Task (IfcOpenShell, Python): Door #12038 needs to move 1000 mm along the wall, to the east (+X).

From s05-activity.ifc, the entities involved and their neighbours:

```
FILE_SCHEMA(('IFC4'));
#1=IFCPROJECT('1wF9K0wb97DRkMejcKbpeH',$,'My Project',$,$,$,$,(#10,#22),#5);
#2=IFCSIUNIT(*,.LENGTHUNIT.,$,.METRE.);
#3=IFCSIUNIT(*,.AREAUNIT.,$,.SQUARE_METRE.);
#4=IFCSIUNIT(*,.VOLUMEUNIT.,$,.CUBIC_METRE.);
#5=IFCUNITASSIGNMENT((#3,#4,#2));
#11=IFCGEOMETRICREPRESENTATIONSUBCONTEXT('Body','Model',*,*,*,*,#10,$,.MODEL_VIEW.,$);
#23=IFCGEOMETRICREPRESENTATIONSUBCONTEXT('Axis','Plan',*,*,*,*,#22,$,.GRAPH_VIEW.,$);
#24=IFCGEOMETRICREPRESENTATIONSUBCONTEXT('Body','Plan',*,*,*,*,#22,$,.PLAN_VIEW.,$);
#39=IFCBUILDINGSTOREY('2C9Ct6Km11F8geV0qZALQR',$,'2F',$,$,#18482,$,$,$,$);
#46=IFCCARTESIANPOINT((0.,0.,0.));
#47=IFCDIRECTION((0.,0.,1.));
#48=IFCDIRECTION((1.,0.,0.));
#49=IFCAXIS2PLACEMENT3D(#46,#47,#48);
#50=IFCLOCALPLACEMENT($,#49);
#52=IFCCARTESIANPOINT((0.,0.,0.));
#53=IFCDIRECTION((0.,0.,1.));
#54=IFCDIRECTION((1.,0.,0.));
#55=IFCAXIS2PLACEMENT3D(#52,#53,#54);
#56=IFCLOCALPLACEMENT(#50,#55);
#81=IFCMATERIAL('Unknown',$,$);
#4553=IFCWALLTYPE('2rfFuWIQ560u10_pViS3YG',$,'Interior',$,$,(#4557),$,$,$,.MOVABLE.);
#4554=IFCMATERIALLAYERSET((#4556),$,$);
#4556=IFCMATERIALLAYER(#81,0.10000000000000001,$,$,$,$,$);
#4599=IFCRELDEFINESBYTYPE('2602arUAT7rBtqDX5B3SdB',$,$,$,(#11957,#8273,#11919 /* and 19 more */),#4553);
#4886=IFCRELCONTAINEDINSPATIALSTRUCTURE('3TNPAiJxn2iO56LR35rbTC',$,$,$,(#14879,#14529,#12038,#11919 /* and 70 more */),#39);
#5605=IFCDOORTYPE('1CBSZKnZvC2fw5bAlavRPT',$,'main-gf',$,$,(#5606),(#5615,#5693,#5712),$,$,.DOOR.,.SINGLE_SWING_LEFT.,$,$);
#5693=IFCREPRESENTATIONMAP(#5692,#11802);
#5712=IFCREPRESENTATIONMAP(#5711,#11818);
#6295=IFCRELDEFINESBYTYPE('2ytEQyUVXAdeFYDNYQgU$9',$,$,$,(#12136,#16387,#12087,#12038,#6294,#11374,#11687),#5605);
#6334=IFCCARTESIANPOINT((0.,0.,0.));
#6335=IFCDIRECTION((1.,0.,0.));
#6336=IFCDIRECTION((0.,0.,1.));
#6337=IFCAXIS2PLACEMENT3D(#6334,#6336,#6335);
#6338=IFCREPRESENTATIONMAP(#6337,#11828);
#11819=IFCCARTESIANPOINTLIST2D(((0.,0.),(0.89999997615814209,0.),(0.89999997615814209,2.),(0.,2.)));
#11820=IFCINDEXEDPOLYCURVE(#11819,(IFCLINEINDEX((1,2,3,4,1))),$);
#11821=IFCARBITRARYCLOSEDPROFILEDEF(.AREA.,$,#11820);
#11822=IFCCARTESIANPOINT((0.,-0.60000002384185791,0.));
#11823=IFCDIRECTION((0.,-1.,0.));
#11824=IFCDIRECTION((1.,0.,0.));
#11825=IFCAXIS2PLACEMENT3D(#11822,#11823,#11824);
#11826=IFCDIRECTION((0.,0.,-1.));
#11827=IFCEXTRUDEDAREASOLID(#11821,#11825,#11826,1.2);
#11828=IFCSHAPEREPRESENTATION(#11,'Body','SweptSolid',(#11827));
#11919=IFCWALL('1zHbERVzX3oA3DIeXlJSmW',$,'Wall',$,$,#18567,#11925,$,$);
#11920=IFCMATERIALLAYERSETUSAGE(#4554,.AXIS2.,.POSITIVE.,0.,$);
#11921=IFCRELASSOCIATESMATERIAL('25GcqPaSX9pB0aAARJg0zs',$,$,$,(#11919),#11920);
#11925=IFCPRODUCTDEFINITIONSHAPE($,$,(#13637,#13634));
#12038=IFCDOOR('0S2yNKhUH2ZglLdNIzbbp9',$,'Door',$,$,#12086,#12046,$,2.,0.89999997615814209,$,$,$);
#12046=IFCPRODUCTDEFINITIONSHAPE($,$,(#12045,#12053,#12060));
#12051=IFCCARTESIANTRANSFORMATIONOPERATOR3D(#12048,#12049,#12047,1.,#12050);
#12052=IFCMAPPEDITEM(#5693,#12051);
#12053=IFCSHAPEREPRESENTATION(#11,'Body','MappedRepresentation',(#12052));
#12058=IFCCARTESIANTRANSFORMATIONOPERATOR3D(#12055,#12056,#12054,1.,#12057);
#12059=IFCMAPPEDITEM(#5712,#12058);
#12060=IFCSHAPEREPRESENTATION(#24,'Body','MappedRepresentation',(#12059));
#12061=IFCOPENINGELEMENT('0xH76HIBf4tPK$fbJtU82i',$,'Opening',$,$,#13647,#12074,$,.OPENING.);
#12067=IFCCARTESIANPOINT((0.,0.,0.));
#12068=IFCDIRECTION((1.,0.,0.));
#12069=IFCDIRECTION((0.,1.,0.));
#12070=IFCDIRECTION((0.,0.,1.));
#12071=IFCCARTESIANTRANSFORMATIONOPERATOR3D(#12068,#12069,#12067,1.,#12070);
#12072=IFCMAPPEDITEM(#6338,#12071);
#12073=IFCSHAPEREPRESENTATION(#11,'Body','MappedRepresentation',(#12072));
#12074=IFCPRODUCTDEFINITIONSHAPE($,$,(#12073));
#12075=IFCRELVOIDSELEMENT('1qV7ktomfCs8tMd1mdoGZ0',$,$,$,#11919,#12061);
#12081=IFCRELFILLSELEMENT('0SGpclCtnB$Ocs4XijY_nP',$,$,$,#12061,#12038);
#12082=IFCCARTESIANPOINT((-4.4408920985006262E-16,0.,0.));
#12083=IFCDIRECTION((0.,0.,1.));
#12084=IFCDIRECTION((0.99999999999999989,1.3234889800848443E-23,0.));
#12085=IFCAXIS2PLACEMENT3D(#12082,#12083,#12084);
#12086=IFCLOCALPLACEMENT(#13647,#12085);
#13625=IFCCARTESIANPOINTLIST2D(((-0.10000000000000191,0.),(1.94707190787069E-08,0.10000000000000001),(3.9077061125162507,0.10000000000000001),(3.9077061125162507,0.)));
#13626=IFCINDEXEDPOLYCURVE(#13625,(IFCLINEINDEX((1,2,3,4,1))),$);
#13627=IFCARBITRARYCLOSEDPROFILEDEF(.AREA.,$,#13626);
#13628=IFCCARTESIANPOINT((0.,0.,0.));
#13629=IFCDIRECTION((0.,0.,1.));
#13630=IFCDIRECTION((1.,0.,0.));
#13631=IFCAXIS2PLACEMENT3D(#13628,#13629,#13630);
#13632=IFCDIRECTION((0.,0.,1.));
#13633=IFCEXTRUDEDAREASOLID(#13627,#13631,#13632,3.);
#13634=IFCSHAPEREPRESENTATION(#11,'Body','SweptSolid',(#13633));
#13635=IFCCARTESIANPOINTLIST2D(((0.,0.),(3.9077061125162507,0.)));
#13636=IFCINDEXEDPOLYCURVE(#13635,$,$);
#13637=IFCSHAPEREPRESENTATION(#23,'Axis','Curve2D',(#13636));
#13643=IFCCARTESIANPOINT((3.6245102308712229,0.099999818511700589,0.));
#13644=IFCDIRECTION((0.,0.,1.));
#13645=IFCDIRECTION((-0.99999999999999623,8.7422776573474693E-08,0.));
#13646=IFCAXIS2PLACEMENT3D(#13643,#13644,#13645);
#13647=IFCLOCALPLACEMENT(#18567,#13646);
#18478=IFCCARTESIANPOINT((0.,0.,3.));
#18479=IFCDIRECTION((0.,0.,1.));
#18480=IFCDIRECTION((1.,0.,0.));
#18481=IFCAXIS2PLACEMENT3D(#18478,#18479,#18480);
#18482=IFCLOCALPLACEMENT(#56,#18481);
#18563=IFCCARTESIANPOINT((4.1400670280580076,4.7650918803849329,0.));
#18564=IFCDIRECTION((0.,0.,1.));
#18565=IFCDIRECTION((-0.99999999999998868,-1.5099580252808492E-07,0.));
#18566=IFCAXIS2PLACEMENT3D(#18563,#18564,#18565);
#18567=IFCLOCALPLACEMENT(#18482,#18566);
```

```python
import ifcopenshell
import ifcopenshell.api.geometry
import ifcopenshell.util.placement

model = ifcopenshell.open("s05-activity.ifc")

door = model.by_guid("0S2yNKhUH2ZglLdNIzbbp9")
opening = door.FillsVoids[0].RelatingOpeningElement
wall = opening.VoidsElements[0].RelatingBuildingElement

wall_matrix = ifcopenshell.util.placement.get_local_placement(wall.ObjectPlacement)
shift = wall_matrix[:3, 0] * -1.0
before = ifcopenshell.util.placement.get_local_placement(door.ObjectPlacement)[:3, 3].copy()

# The door is placed relative to its opening, so it follows when the opening moves.
matrix = ifcopenshell.util.placement.get_local_placement(opening.ObjectPlacement)
matrix[:3, 3] += shift
ifcopenshell.api.geometry.edit_object_placement(
    model, product=opening, matrix=matrix, is_si=False, should_transform_children=True
)

after = ifcopenshell.util.placement.get_local_placement(door.ObjectPlacement)[:3, 3]
print("door moved by", (after - before).round(3) + 0.0)

model.write("s05-activity-out.ifc")
```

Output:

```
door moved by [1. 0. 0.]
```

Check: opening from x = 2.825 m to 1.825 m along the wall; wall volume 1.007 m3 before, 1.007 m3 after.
